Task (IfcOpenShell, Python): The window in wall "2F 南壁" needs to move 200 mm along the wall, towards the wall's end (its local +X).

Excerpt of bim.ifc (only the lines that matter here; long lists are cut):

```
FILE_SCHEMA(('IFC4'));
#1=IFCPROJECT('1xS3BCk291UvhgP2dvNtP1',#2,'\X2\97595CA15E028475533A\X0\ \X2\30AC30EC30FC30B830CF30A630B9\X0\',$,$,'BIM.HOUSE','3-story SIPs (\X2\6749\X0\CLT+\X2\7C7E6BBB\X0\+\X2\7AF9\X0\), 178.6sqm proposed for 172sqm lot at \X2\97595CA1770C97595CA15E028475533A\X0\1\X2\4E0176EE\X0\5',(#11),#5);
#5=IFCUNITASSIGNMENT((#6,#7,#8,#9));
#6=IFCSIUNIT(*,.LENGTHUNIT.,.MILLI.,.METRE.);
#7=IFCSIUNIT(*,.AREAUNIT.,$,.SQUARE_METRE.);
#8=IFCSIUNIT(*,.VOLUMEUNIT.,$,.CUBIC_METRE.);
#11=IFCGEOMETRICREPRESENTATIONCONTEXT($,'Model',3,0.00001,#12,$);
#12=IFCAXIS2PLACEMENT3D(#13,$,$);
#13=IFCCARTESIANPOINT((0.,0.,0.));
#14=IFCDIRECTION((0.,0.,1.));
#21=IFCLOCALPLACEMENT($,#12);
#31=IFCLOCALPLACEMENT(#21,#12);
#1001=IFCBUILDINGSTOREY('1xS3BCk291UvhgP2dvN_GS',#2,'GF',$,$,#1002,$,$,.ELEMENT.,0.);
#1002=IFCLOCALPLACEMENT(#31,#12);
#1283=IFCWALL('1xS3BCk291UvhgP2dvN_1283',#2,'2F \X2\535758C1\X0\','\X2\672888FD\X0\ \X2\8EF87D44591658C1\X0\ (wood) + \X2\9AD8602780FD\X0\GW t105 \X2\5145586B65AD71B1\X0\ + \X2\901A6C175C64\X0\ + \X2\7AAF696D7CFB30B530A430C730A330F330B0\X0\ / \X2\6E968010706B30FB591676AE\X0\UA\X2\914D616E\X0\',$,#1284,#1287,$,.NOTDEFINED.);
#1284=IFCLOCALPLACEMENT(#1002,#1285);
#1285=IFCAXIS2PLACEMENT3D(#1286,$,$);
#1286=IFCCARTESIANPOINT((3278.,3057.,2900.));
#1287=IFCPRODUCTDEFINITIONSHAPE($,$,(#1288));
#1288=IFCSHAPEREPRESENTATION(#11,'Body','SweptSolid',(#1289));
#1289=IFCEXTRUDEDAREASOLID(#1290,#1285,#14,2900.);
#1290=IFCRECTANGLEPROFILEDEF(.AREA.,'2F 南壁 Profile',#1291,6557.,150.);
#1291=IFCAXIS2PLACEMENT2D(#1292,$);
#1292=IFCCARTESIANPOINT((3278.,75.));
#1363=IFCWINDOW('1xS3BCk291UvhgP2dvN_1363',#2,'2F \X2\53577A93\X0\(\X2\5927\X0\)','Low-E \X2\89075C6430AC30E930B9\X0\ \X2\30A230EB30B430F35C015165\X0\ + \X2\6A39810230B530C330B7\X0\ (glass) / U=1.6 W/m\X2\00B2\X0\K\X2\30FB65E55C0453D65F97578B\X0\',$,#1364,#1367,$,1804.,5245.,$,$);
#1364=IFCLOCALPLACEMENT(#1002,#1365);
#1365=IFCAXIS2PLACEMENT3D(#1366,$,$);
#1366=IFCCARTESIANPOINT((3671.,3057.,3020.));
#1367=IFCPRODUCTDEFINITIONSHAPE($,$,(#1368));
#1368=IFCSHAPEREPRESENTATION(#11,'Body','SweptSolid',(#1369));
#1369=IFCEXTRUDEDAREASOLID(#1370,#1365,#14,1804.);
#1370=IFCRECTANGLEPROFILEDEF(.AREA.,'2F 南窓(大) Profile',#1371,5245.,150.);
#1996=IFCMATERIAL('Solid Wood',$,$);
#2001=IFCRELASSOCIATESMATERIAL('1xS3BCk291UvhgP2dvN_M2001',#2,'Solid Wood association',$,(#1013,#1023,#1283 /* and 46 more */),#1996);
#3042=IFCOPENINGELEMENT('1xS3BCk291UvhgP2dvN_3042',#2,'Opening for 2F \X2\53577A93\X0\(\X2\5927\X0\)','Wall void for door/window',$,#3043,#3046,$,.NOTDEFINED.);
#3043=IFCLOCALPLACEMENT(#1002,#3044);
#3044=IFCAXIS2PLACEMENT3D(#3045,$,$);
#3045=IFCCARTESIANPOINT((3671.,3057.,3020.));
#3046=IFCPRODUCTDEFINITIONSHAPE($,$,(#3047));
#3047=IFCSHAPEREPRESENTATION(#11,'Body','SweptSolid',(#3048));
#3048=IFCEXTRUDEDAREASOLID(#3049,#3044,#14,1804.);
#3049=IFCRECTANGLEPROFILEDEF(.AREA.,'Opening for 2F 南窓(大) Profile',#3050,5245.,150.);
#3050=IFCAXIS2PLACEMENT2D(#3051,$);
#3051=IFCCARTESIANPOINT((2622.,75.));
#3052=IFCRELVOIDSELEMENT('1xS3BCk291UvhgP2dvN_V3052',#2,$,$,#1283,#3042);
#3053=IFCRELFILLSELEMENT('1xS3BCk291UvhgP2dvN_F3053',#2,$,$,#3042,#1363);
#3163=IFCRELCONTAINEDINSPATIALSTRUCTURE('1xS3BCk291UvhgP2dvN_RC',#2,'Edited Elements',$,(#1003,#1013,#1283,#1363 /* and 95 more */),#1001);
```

```python
import ifcopenshell
import ifcopenshell.api.geometry
import ifcopenshell.util.placement
import ifcopenshell.util.unit

model = ifcopenshell.open("bim.ifc")
unit_scale = ifcopenshell.util.unit.calculate_unit_scale(model)

window = model.by_id(1363)
opening = window.FillsVoids[0].RelatingOpeningElement
wall = opening.VoidsElements[0].RelatingBuildingElement

wall_matrix = ifcopenshell.util.placement.get_local_placement(wall.ObjectPlacement)
shift = wall_matrix[:3, 0] * 0.2 / unit_scale
before = ifcopenshell.util.placement.get_local_placement(window.ObjectPlacement)[:3, 3].copy()

# The window is not placed relative to its opening, so move both.
for product in (opening, window):
    matrix = ifcopenshell.util.placement.get_local_placement(product.ObjectPlacement)
    matrix[:3, 3] += shift
    ifcopenshell.api.geometry.edit_object_placement(model, product=product, matrix=matrix, is_si=False)

after = ifcopenshell.util.placement.get_local_placement(window.ObjectPlacement)[:3, 3]
print("window moved by", (after - before).round(3) + 0.0)

model.write("bim_edited.ifc")
```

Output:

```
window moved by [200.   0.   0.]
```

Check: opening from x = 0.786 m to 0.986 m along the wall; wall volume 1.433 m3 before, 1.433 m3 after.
